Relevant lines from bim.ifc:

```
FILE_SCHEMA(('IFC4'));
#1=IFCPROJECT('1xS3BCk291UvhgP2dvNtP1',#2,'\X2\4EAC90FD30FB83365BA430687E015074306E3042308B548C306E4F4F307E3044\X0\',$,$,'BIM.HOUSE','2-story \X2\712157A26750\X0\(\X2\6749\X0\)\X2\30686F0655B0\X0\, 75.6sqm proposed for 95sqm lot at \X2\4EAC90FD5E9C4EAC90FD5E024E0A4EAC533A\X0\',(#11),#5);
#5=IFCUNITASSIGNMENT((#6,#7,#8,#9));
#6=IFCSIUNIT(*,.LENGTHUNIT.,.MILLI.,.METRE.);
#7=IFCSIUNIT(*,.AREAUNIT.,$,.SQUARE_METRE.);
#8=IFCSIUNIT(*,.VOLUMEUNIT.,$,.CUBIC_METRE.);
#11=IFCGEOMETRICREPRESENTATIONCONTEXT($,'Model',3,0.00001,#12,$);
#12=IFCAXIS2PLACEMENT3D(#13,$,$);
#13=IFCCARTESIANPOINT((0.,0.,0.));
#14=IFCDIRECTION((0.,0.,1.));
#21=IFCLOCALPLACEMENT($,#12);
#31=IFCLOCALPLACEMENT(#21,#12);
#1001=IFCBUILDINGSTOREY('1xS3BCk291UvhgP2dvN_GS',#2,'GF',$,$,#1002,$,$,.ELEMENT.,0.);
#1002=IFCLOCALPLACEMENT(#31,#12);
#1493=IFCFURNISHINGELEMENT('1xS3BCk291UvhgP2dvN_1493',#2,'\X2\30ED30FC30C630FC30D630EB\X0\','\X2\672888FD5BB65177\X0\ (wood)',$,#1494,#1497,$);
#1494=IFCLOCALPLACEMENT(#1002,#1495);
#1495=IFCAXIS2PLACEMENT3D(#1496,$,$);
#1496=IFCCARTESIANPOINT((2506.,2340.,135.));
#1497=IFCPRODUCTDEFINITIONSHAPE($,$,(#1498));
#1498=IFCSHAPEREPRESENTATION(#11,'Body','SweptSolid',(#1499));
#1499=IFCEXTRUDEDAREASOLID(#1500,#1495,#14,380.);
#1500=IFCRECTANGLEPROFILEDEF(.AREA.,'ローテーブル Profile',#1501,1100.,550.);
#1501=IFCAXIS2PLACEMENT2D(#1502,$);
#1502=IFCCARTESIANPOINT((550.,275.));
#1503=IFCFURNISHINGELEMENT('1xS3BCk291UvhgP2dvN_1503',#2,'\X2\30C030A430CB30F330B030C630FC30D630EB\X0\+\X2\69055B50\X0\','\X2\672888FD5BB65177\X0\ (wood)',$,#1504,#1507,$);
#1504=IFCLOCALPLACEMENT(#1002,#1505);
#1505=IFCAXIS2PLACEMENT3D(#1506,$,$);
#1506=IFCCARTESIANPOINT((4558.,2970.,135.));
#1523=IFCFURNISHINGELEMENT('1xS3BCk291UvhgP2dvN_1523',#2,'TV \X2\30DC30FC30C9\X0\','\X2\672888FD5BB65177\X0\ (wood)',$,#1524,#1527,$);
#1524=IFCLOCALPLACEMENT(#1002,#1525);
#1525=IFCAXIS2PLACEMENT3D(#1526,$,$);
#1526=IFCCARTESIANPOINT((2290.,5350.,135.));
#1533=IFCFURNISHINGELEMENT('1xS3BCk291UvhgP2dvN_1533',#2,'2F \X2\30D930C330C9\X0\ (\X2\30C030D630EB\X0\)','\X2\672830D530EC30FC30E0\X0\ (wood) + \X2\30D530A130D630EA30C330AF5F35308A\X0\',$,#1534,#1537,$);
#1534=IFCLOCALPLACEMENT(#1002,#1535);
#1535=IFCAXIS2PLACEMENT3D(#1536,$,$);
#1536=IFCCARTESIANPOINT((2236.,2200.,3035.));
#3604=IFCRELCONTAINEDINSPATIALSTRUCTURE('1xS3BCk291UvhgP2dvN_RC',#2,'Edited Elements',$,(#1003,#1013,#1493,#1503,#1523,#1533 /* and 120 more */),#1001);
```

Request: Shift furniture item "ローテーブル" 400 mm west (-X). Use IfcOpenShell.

```python
import ifcopenshell
import ifcopenshell.api.geometry
import ifcopenshell.util.placement
import ifcopenshell.util.unit

model = ifcopenshell.open("bim.ifc")
unit_scale = ifcopenshell.util.unit.calculate_unit_scale(model)

item = model.by_guid("1xS3BCk291UvhgP2dvN_1493")
matrix = ifcopenshell.util.placement.get_local_placement(item.ObjectPlacement)
matrix[0, 3] -= 0.4 / unit_scale
ifcopenshell.api.geometry.edit_object_placement(model, product=item, matrix=matrix, is_si=False)

print(ifcopenshell.util.placement.get_local_placement(item.ObjectPlacement).round(3) + 0.0)

model.write("bim_edited.ifc")
```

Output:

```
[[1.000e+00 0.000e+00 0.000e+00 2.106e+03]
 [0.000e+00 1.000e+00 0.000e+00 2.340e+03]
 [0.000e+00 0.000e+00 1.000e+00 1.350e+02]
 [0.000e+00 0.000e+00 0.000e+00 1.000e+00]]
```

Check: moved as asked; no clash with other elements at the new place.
